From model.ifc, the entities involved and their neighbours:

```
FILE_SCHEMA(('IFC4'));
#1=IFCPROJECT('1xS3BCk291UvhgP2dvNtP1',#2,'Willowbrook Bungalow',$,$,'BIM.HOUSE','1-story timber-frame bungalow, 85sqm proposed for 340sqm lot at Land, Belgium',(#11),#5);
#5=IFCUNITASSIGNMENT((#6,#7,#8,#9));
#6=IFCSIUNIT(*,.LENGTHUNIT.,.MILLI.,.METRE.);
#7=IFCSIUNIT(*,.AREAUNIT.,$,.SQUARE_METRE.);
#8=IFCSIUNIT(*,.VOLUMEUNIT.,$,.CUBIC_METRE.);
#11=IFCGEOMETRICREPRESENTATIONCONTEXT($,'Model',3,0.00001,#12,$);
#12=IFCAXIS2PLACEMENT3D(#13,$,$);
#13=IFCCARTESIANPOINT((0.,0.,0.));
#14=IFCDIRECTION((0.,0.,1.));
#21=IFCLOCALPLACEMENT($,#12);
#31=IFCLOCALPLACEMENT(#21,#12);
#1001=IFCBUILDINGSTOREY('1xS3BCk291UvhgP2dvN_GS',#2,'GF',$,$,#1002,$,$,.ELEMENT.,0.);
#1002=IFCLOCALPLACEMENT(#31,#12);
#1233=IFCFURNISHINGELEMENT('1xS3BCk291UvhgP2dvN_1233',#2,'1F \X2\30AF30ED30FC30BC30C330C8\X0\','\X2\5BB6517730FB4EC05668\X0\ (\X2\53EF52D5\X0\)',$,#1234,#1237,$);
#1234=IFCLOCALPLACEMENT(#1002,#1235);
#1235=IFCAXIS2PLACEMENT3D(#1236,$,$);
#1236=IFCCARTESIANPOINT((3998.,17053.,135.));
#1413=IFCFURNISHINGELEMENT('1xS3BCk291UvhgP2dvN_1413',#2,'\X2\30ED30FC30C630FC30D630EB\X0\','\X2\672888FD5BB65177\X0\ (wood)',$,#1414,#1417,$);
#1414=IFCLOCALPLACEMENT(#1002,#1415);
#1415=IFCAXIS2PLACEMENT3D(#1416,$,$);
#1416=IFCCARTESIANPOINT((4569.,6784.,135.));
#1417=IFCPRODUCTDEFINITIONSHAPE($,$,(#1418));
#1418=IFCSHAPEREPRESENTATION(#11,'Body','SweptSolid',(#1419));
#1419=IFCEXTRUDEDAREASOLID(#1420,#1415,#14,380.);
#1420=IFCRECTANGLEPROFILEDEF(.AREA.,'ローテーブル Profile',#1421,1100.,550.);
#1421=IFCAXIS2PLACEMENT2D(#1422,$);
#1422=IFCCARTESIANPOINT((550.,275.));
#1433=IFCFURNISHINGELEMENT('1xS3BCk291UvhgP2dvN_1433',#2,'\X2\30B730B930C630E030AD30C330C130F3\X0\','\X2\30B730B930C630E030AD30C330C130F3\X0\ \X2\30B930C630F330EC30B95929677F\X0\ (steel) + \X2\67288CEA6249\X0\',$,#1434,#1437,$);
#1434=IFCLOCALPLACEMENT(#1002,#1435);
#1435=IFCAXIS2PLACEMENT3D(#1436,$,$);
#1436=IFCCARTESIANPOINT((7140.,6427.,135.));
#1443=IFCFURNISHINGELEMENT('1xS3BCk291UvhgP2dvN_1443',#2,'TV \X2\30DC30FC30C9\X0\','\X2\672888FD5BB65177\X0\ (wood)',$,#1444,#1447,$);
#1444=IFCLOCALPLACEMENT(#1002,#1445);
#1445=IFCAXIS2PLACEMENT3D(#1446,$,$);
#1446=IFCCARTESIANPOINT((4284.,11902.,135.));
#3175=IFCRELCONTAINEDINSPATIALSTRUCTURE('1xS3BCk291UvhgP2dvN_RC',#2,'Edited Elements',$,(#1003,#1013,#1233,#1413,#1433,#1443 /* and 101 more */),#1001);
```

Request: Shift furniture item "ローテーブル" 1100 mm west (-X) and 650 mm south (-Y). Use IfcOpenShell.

```python
import ifcopenshell
import ifcopenshell.api.geometry
import ifcopenshell.util.placement
import ifcopenshell.util.unit

model = ifcopenshell.open("model.ifc")
unit_scale = ifcopenshell.util.unit.calculate_unit_scale(model)

item = model.by_id(1413)
matrix = ifcopenshell.util.placement.get_local_placement(item.ObjectPlacement)
matrix[0, 3] -= 1.1 / unit_scale
matrix[1, 3] -= 0.65 / unit_scale
ifcopenshell.api.geometry.edit_object_placement(model, product=item, matrix=matrix, is_si=False)

print(ifcopenshell.util.placement.get_local_placement(item.ObjectPlacement).round(3) + 0.0)

model.write("model_rev.ifc")
```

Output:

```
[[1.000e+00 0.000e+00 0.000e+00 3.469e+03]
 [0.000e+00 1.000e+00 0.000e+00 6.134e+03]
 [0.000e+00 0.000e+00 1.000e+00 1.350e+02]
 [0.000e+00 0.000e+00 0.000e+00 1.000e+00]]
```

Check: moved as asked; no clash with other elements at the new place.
